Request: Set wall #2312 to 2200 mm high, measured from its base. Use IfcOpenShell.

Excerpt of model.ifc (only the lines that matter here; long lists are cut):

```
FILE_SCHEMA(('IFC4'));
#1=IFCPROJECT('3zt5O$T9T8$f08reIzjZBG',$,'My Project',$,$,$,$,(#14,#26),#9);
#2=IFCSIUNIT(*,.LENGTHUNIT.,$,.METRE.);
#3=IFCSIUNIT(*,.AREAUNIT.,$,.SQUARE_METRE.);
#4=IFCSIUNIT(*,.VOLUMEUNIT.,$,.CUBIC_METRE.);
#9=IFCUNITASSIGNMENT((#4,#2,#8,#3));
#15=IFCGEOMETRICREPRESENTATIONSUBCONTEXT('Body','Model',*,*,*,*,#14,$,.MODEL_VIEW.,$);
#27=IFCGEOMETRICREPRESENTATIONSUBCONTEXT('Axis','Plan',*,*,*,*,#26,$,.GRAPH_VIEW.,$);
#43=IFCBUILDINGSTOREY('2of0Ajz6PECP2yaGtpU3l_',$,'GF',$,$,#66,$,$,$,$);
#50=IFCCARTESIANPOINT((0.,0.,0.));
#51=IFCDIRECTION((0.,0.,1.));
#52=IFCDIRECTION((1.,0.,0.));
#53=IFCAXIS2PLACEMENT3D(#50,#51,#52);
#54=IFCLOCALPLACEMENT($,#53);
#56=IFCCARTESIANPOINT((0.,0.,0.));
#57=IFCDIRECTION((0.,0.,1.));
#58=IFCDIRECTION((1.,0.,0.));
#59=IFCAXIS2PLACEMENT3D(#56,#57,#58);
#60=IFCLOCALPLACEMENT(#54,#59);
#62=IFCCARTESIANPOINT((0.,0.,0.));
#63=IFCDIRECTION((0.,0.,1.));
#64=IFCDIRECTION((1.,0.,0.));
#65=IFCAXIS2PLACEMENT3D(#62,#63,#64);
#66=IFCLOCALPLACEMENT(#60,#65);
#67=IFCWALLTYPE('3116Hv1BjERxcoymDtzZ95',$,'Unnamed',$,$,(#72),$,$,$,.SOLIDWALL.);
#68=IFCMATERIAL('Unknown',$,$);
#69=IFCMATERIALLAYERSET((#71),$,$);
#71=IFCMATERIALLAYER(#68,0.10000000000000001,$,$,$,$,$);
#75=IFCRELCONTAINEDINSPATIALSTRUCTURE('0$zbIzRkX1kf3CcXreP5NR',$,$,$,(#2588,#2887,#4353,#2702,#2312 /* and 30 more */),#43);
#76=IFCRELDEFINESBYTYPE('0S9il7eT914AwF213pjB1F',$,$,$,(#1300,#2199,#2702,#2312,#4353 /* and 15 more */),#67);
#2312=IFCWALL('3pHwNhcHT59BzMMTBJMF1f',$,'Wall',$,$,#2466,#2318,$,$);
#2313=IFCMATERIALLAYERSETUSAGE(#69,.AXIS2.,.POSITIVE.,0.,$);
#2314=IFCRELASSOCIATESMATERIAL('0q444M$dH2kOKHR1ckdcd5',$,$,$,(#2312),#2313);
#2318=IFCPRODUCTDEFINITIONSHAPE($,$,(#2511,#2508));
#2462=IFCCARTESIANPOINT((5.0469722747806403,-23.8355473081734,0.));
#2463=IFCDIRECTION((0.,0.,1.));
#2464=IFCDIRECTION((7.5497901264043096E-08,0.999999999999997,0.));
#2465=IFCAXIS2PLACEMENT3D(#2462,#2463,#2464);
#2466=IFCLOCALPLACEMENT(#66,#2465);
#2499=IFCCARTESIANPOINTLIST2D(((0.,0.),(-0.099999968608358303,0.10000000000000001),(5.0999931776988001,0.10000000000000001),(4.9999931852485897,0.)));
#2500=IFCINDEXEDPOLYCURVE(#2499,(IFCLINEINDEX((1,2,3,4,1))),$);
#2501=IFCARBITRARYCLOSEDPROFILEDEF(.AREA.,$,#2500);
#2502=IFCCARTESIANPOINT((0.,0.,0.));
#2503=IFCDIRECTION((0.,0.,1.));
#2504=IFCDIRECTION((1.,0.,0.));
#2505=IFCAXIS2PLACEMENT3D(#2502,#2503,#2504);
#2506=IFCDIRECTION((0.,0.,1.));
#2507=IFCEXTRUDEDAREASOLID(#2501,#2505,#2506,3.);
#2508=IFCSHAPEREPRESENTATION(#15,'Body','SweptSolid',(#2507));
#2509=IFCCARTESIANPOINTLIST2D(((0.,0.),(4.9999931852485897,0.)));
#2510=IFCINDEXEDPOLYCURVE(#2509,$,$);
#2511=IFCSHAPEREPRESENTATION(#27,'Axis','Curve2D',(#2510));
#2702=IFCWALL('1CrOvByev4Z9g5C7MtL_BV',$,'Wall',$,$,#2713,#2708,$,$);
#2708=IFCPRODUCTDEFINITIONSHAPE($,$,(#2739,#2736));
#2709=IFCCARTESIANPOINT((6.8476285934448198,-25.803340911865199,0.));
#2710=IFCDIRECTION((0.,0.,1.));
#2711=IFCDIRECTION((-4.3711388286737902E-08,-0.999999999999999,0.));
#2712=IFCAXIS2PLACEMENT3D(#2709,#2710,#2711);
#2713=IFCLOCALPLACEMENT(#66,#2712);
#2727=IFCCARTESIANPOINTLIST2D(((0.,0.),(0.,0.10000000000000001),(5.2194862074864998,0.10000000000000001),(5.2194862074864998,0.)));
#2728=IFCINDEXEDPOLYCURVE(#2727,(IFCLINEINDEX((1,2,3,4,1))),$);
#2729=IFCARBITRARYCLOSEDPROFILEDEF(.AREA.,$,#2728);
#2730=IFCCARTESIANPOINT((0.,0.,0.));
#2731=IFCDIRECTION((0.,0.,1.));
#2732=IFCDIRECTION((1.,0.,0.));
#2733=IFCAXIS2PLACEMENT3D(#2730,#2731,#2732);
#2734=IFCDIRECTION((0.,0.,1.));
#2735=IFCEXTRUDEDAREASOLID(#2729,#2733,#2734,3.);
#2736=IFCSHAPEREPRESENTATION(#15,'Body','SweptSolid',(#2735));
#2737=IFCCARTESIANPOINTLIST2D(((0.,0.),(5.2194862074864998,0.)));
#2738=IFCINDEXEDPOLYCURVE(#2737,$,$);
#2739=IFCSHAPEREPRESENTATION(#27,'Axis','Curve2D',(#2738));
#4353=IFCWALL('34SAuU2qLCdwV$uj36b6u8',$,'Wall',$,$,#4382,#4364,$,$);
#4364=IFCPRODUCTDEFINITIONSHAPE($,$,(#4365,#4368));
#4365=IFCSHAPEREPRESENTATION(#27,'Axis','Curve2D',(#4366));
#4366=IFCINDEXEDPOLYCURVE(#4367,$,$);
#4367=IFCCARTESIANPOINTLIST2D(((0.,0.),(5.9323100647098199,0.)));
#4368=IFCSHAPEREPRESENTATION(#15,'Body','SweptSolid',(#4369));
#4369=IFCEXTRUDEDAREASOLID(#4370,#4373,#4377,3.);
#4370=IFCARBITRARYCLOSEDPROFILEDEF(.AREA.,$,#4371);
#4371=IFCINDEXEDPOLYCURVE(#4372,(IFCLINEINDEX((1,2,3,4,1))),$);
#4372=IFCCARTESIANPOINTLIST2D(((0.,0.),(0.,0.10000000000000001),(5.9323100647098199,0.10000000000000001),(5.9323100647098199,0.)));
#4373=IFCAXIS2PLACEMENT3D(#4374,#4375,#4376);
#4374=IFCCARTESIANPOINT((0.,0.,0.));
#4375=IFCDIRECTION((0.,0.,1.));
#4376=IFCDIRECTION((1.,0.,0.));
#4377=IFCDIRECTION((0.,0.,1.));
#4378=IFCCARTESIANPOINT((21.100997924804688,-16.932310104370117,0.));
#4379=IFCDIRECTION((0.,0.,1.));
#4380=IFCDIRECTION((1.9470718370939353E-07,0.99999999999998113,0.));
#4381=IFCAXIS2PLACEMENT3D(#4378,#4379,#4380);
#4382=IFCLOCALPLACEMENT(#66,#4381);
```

```python
import ifcopenshell
import ifcopenshell.geom
import ifcopenshell.util.representation
import ifcopenshell.util.shape

model = ifcopenshell.open("model.ifc")
settings = ifcopenshell.geom.settings()


def volume(element):
    """Net volume in cubic metres, openings subtracted."""
    shape = ifcopenshell.geom.create_shape(settings, element)
    return ifcopenshell.util.shape.get_volume(shape.geometry)


wall = model.by_id(2312)
before = volume(wall)

body = ifcopenshell.util.representation.get_representation(wall, "Model", "Body")
solid = body.Items[0]
old_height = solid.Depth
solid.Depth = 2.2
after = volume(wall)

print(f"height {old_height:g} -> {solid.Depth:g}, volume {before:.3f} -> {after:.3f} m3")

model.write("model_updated.ifc")
```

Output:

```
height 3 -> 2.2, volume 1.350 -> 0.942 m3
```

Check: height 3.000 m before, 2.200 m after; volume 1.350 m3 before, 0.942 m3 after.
